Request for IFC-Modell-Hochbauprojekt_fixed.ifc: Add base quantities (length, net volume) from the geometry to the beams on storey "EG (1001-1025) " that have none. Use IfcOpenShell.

First a look at what the model holds.

```python
import ifcopenshell
import ifcopenshell.util.element
import ifcopenshell.util.unit

model = ifcopenshell.open("IFC-Modell-Hochbauprojekt_fixed.ifc")
print(model.schema)
for unit_type in ("LENGTHUNIT", "AREAUNIT", "VOLUMEUNIT"):
    print(unit_type, ifcopenshell.util.unit.calculate_unit_scale(model, unit_type))
storey = next(s for s in model.by_type("IfcBuildingStorey") if s.Name == "EG (1001-1025) ")
beams = [e for e in ifcopenshell.util.element.get_decomposition(storey) if e.is_a("IfcBeam")]
for e in sorted(beams, key=lambda e: e.id()):
    print(e.id(), e.is_a(), e.Name, list(ifcopenshell.util.element.get_psets(e, qtos_only=True)), sep=" | ")
```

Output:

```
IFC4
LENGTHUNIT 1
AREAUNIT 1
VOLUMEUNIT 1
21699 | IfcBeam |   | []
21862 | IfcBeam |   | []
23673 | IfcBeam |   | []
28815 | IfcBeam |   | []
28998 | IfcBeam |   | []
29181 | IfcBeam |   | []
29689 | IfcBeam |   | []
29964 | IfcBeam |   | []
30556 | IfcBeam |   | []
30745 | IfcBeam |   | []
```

```python
import ifcopenshell
import ifcopenshell.api.pset
import ifcopenshell.geom
import ifcopenshell.util.element
import ifcopenshell.util.shape
import ifcopenshell.util.unit

model = ifcopenshell.open("IFC-Modell-Hochbauprojekt_fixed.ifc")
unit_scale = ifcopenshell.util.unit.calculate_unit_scale(model)
volume_scale = ifcopenshell.util.unit.calculate_unit_scale(model, "VOLUMEUNIT")
settings = ifcopenshell.geom.settings()

storey = next(s for s in model.by_type("IfcBuildingStorey") if s.Name == "EG (1001-1025) ")
beams = [e for e in ifcopenshell.util.element.get_decomposition(storey) if e.is_a("IfcBeam")]

for e in sorted(beams, key=lambda e: e.id()):
    if ifcopenshell.util.element.get_psets(e, qtos_only=True, should_inherit=False):
        continue
    # Geometry comes back in metres, in the element's own axes.
    shape = ifcopenshell.geom.create_shape(settings, e)
    values = {
        "Length": ifcopenshell.util.shape.get_max_xyz(shape.geometry) / unit_scale,
        "NetVolume": ifcopenshell.util.shape.get_volume(shape.geometry) / volume_scale,
    }
    qto = ifcopenshell.api.pset.add_qto(model, product=e, name="Qto_BeamBaseQuantities")
    ifcopenshell.api.pset.edit_qto(model, qto=qto, properties=values)
    print(e.id(), {k: round(v, 3) for k, v in values.items()})

model.write("IFC-Modell-Hochbauprojekt_fixed_rev.ifc")
```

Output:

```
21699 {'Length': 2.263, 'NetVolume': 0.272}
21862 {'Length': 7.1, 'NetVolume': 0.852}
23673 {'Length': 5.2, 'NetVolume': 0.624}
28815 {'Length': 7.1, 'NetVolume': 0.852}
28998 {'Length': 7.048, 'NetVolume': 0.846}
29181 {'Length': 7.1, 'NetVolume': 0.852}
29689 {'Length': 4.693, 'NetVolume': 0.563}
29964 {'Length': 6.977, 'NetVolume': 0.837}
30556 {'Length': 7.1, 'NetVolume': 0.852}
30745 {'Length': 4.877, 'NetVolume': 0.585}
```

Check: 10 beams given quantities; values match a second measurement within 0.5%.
